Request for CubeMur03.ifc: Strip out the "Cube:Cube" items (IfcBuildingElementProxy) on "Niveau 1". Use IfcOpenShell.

First a look at what the model holds.

```python
import ifcopenshell
import ifcopenshell.util.element

model = ifcopenshell.open("CubeMur03.ifc")
print(model.schema)
storey = next(s for s in model.by_type("IfcBuildingStorey") if s.Name == "Niveau 1")
proxies = [e for e in ifcopenshell.util.element.get_decomposition(storey) if e.is_a("IfcBuildingElementProxy")]
seen = {}
for e in proxies:
    element_type = ifcopenshell.util.element.get_type(e)
    name = element_type.Name if element_type not in (None, e) else None
    seen[name] = seen.get(name, 0) + 1
for name, count in sorted(seen.items(), key=str):
    print(count, "x", name)
```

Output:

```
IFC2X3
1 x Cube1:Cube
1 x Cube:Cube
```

```python
import ifcopenshell
import ifcopenshell.api.root
import ifcopenshell.util.element

model = ifcopenshell.open("CubeMur03.ifc")

storey = next(s for s in model.by_type("IfcBuildingStorey") if s.Name == "Niveau 1")
proxies = [e for e in ifcopenshell.util.element.get_decomposition(storey) if e.is_a("IfcBuildingElementProxy")]
targets = [e for e in proxies if (t := ifcopenshell.util.element.get_type(e)) not in (None, e) and t.Name == "Cube:Cube"]

for e in targets:
    ifcopenshell.api.root.remove_product(model, product=e)
print(len(targets), "removed")

model.write("CubeMur03_rev.ifc")
```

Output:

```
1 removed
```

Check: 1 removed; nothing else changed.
